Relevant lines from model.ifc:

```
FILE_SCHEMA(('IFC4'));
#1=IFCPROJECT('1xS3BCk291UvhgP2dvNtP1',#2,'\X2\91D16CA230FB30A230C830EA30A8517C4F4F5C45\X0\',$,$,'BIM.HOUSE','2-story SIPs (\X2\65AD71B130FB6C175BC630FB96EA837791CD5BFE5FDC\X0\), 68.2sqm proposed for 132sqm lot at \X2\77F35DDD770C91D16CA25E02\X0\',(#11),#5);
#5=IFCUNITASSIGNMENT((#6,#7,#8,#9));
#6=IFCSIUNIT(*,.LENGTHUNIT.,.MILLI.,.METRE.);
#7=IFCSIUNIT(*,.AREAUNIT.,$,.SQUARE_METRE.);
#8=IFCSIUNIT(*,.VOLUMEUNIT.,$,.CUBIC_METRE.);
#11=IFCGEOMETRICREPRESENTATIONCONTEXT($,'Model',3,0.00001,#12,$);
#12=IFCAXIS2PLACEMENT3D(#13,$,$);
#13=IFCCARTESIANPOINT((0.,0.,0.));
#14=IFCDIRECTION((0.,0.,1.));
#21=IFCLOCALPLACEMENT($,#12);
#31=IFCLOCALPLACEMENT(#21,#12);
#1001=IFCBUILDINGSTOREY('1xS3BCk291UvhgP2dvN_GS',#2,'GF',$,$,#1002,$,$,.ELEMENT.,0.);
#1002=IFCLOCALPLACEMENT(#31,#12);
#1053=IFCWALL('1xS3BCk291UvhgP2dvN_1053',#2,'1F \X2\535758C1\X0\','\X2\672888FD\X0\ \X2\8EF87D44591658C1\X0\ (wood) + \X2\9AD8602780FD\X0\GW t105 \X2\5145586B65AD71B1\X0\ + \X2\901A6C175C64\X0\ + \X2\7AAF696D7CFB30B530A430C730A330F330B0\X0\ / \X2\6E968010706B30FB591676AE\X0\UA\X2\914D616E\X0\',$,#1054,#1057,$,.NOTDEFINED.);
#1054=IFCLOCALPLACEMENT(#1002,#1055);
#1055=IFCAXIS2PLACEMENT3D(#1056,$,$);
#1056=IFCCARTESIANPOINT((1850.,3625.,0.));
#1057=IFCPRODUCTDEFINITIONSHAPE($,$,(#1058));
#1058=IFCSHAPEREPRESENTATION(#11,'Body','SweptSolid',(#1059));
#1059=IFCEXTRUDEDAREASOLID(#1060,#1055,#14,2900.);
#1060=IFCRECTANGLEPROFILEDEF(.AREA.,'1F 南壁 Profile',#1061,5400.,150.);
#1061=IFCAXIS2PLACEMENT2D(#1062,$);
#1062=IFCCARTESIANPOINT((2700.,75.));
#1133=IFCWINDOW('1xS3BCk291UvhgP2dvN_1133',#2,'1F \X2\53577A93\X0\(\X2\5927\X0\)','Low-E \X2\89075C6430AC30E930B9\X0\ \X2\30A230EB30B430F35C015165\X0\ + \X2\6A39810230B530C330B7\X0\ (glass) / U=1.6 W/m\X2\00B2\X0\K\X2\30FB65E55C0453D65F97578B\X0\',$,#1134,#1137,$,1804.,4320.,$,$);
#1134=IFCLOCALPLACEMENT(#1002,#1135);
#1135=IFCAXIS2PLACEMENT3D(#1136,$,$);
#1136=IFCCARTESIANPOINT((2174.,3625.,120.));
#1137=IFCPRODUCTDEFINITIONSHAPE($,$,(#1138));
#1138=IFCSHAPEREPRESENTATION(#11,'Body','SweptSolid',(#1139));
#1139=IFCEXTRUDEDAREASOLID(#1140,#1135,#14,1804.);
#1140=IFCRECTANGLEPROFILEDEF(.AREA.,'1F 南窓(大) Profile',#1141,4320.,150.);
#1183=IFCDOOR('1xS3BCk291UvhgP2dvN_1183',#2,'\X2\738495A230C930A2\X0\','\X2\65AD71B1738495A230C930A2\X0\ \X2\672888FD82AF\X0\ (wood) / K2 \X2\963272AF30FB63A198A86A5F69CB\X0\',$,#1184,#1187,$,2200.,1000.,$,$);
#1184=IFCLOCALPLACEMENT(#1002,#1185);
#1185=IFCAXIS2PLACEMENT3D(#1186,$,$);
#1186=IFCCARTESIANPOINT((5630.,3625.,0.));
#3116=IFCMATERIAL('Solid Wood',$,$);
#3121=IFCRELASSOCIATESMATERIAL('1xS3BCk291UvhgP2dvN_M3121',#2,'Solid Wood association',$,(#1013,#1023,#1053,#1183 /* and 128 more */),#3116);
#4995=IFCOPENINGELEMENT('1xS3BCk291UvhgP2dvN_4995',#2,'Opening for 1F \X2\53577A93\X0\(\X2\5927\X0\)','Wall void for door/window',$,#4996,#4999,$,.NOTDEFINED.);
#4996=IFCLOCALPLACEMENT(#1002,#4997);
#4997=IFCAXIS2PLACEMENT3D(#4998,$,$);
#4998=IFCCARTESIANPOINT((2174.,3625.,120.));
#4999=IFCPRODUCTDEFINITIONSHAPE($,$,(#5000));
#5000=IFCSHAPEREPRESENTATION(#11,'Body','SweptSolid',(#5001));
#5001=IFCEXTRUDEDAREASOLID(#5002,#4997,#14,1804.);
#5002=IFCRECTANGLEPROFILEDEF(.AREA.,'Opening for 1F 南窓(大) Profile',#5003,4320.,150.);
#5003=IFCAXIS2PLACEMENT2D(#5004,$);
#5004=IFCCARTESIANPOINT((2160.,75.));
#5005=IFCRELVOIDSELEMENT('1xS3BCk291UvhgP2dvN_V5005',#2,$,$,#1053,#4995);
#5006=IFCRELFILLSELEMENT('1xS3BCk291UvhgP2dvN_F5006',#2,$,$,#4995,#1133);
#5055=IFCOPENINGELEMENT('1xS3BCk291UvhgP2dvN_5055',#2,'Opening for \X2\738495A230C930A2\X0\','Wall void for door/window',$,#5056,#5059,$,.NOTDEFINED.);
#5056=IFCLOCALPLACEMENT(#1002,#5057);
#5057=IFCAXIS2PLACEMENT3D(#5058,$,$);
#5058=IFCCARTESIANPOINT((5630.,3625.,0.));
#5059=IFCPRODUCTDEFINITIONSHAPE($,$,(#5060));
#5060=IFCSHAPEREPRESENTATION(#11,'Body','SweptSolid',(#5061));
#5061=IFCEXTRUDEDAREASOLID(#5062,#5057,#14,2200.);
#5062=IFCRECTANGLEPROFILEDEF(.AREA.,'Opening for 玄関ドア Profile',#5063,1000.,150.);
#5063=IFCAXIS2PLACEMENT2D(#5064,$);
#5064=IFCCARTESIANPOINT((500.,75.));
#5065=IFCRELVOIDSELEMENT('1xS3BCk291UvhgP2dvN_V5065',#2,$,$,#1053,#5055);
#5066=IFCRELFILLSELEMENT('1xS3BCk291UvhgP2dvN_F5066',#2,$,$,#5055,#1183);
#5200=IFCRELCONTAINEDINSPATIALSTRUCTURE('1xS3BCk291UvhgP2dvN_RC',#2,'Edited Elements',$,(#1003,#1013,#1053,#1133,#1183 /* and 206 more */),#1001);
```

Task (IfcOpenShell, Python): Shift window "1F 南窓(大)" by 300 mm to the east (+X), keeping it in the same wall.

```python
import ifcopenshell
import ifcopenshell.api.geometry
import ifcopenshell.util.placement
import ifcopenshell.util.unit

model = ifcopenshell.open("model.ifc")
unit_scale = ifcopenshell.util.unit.calculate_unit_scale(model)

window = model.by_guid("1xS3BCk291UvhgP2dvN_1133")
opening = window.FillsVoids[0].RelatingOpeningElement
wall = opening.VoidsElements[0].RelatingBuildingElement

wall_matrix = ifcopenshell.util.placement.get_local_placement(wall.ObjectPlacement)
shift = wall_matrix[:3, 0] * 0.3 / unit_scale
before = ifcopenshell.util.placement.get_local_placement(window.ObjectPlacement)[:3, 3].copy()

# The window is not placed relative to its opening, so move both.
for product in (opening, window):
    matrix = ifcopenshell.util.placement.get_local_placement(product.ObjectPlacement)
    matrix[:3, 3] += shift
    ifcopenshell.api.geometry.edit_object_placement(model, product=product, matrix=matrix, is_si=False)

after = ifcopenshell.util.placement.get_local_placement(window.ObjectPlacement)[:3, 3]
print("window moved by", (after - before).round(3) + 0.0)

model.write("model_edited.ifc")
```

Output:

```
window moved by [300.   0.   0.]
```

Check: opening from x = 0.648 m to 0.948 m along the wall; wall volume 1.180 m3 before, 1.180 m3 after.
